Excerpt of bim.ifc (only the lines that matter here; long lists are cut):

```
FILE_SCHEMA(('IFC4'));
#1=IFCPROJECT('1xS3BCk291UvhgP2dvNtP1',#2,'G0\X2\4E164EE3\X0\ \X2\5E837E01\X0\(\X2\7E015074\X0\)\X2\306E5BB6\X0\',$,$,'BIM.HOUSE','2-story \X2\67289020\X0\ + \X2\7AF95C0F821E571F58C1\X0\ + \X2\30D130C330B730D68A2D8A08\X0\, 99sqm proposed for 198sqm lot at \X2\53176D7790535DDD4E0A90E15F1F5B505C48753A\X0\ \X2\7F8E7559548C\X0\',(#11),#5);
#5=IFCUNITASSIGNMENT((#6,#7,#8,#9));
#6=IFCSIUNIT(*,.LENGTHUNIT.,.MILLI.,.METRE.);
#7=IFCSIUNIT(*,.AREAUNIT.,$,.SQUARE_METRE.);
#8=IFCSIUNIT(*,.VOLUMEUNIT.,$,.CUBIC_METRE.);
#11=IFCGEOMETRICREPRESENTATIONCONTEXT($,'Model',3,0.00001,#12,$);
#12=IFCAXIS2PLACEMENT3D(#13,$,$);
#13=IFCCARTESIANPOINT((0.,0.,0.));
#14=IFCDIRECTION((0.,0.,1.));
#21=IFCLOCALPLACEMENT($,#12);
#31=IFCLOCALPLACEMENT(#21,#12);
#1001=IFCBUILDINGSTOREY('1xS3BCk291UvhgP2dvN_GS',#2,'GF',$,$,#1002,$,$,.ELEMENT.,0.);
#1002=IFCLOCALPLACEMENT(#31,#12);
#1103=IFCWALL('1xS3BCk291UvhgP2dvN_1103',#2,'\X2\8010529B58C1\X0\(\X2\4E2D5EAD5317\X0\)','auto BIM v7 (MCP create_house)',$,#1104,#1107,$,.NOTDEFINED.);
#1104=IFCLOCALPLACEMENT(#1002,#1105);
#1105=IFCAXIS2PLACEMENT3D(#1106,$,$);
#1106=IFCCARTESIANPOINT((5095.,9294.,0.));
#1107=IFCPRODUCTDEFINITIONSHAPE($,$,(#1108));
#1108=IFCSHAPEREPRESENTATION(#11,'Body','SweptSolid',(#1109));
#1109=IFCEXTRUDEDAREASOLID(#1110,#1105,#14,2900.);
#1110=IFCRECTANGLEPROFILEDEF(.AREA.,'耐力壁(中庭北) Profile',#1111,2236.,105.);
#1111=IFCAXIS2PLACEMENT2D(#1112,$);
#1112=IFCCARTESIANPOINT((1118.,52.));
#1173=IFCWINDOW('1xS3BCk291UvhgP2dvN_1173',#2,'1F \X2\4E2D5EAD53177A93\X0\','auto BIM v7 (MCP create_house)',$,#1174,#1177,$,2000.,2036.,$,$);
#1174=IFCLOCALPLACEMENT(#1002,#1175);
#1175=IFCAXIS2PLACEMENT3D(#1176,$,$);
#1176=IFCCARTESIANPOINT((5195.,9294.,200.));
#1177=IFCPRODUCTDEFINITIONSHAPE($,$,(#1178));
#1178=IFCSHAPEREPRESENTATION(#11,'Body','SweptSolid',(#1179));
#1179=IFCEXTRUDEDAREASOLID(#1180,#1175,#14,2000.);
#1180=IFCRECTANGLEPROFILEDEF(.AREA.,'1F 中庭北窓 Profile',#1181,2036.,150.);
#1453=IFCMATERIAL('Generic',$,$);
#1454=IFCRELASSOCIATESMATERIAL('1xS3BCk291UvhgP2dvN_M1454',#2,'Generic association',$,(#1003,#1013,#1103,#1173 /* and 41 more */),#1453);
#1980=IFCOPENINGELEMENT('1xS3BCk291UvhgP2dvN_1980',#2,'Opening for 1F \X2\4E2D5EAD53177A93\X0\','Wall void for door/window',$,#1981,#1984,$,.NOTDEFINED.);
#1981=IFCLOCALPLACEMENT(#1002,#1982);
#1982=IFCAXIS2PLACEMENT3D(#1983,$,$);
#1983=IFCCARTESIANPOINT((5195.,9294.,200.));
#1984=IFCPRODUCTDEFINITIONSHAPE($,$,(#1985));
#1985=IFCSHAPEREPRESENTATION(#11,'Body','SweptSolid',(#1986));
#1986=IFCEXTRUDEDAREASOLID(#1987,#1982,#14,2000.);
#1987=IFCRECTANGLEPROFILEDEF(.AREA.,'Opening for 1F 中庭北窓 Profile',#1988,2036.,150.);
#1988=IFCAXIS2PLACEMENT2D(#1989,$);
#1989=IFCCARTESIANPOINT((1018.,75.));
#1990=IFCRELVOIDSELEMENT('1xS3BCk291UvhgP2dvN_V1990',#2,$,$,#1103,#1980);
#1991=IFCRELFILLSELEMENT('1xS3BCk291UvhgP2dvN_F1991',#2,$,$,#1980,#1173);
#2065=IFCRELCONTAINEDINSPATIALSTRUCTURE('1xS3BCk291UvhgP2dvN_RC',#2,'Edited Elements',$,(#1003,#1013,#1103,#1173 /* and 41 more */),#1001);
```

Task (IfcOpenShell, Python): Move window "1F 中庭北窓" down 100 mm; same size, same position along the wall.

```python
import numpy as np
import ifcopenshell
import ifcopenshell.api.geometry
import ifcopenshell.util.placement
import ifcopenshell.util.unit

model = ifcopenshell.open("bim.ifc")
unit_scale = ifcopenshell.util.unit.calculate_unit_scale(model)

window = model.by_guid("1xS3BCk291UvhgP2dvN_1173")
opening = window.FillsVoids[0].RelatingOpeningElement
dz = -0.1 / unit_scale

shift = np.array([0.0, 0.0, dz])
# The window is not placed relative to its opening, so move both.
for product in (opening, window):
    matrix = ifcopenshell.util.placement.get_local_placement(product.ObjectPlacement)
    matrix[:3, 3] += shift
    ifcopenshell.api.geometry.edit_object_placement(model, product=product, matrix=matrix, is_si=False)

print(f"moved by {dz * unit_scale:+.3f} m")

model.write("bim_updated.ifc")
```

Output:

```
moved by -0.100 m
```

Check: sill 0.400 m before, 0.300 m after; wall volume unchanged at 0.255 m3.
